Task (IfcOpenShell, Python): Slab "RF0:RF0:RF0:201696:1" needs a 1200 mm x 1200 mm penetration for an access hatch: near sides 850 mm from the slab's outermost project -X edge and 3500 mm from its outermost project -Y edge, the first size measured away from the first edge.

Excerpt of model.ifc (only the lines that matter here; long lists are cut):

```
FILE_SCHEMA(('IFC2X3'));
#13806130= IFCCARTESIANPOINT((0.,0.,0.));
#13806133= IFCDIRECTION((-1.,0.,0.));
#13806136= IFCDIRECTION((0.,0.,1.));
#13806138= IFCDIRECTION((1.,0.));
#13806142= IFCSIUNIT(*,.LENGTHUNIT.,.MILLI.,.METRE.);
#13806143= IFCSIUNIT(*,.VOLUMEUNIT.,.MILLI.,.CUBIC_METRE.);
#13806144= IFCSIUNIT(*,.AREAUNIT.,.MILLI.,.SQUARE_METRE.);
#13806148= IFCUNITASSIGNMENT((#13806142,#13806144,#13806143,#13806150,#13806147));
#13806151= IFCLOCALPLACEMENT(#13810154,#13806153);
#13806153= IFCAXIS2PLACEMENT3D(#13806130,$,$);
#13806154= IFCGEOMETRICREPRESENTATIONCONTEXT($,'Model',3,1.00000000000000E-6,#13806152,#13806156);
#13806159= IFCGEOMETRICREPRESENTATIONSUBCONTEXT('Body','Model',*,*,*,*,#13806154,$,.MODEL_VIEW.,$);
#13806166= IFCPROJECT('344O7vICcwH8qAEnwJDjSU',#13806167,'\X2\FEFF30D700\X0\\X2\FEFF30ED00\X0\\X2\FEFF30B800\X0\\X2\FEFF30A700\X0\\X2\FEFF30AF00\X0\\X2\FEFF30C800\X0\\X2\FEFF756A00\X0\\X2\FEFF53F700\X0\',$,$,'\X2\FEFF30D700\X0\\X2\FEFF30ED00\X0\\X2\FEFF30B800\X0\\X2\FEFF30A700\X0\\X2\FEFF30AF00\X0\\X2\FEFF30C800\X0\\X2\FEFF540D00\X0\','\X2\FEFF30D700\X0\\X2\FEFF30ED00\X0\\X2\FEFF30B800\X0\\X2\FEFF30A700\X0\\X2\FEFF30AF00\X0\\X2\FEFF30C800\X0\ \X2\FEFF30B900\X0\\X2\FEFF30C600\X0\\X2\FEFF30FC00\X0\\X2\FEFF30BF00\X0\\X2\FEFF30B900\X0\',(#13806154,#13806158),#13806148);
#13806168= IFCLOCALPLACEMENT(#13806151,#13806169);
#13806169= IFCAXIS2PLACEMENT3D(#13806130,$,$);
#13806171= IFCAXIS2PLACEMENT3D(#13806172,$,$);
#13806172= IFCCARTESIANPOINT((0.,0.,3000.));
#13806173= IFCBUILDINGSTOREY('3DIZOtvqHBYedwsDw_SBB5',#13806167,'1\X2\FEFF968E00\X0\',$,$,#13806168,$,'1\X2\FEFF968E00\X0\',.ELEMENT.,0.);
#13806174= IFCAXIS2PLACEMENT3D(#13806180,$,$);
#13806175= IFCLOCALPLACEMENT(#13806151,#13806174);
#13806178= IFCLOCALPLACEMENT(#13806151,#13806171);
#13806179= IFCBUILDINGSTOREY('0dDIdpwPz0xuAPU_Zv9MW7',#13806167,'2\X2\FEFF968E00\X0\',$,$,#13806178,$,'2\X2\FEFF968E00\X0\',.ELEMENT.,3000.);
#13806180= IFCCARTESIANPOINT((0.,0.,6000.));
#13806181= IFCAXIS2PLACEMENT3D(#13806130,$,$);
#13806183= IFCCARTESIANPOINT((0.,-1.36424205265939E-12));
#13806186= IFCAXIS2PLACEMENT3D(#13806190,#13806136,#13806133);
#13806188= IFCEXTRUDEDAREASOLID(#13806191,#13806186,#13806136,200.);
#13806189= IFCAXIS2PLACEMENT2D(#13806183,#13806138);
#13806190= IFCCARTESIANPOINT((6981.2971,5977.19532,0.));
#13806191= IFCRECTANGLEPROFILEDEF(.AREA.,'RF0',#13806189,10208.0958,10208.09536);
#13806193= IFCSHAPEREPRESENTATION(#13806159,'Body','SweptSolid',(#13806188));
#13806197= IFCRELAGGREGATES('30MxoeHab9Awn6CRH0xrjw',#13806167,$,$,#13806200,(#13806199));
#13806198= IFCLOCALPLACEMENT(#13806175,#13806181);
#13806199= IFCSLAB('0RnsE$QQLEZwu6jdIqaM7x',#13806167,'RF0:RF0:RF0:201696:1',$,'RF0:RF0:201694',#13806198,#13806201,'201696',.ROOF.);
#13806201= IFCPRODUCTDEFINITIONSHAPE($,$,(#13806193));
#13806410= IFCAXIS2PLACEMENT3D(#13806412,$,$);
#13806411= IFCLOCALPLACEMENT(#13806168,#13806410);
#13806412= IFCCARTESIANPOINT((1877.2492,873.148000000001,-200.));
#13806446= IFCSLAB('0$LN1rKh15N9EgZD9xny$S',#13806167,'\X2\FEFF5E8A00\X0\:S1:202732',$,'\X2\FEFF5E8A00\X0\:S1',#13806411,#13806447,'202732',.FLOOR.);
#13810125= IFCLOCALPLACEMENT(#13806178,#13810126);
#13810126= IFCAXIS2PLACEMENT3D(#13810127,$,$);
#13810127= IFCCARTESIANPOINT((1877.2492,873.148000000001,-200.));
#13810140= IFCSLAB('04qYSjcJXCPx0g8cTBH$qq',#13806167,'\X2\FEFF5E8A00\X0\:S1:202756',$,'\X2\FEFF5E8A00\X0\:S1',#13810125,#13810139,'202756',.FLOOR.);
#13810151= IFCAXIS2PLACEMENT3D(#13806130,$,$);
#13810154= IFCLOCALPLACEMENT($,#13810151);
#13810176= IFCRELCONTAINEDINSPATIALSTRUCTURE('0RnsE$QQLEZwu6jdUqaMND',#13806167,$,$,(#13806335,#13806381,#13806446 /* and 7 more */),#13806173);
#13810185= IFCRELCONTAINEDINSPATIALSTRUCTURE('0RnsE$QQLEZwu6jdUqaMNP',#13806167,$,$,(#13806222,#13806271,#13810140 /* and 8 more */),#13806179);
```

```python
import numpy as np
import ifcopenshell
import ifcopenshell.api.feature
import ifcopenshell.api.geometry
import ifcopenshell.api.root
import ifcopenshell.geom
import ifcopenshell.util.placement
import ifcopenshell.util.representation
import ifcopenshell.util.shape
import ifcopenshell.util.unit

model = ifcopenshell.open("model.ifc")
unit_scale = ifcopenshell.util.unit.calculate_unit_scale(model)
settings = ifcopenshell.geom.settings()


def volume(element):
    """Net volume in cubic metres, openings subtracted."""
    shape = ifcopenshell.geom.create_shape(settings, element)
    return ifcopenshell.util.shape.get_volume(shape.geometry)


slab = model.by_guid("0RnsE$QQLEZwu6jdIqaM7x")
before = volume(slab)

# Extent in the slab's own axes, in metres. The edges named are its -X and -Y sides.
slab_shape = ifcopenshell.geom.create_shape(settings, slab)
vertices = ifcopenshell.util.shape.get_vertices(slab_shape.geometry)
x_min, y_min, bottom = vertices.min(axis=0)
top = vertices[:, 2].max()

opening = ifcopenshell.api.root.create_entity(model, ifc_class="IfcOpeningElement", name="Access hatch opening")
context = ifcopenshell.util.representation.get_context(model, "Model", "Body", "MODEL_VIEW")
width, depth = 1.2, 1.2
outline = [(0.0, 0.0), (width, 0.0), (width, depth), (0.0, depth), (0.0, 0.0)]
# Overshoot both faces by 50 mm so the cut is clean.
shape = ifcopenshell.api.geometry.add_slab_representation(
    model, context=context, depth=top - bottom + 0.1, polyline=outline
)
ifcopenshell.api.geometry.assign_representation(model, product=opening, representation=shape)

matrix = ifcopenshell.util.placement.get_local_placement(slab.ObjectPlacement)
matrix[:, 3] = matrix @ np.append(np.array([x_min + 0.85, y_min + 3.5, bottom - 0.05]) / unit_scale, 1.0)
ifcopenshell.api.geometry.edit_object_placement(model, product=opening, matrix=matrix, is_si=False)
ifcopenshell.api.feature.add_feature(model, feature=opening, element=slab)

after = volume(slab)

print(f"slab volume {before:.3f} -> {after:.3f} m3")

model.write("model-out.ifc")
```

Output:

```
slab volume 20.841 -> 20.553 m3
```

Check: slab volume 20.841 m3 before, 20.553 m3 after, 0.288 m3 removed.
